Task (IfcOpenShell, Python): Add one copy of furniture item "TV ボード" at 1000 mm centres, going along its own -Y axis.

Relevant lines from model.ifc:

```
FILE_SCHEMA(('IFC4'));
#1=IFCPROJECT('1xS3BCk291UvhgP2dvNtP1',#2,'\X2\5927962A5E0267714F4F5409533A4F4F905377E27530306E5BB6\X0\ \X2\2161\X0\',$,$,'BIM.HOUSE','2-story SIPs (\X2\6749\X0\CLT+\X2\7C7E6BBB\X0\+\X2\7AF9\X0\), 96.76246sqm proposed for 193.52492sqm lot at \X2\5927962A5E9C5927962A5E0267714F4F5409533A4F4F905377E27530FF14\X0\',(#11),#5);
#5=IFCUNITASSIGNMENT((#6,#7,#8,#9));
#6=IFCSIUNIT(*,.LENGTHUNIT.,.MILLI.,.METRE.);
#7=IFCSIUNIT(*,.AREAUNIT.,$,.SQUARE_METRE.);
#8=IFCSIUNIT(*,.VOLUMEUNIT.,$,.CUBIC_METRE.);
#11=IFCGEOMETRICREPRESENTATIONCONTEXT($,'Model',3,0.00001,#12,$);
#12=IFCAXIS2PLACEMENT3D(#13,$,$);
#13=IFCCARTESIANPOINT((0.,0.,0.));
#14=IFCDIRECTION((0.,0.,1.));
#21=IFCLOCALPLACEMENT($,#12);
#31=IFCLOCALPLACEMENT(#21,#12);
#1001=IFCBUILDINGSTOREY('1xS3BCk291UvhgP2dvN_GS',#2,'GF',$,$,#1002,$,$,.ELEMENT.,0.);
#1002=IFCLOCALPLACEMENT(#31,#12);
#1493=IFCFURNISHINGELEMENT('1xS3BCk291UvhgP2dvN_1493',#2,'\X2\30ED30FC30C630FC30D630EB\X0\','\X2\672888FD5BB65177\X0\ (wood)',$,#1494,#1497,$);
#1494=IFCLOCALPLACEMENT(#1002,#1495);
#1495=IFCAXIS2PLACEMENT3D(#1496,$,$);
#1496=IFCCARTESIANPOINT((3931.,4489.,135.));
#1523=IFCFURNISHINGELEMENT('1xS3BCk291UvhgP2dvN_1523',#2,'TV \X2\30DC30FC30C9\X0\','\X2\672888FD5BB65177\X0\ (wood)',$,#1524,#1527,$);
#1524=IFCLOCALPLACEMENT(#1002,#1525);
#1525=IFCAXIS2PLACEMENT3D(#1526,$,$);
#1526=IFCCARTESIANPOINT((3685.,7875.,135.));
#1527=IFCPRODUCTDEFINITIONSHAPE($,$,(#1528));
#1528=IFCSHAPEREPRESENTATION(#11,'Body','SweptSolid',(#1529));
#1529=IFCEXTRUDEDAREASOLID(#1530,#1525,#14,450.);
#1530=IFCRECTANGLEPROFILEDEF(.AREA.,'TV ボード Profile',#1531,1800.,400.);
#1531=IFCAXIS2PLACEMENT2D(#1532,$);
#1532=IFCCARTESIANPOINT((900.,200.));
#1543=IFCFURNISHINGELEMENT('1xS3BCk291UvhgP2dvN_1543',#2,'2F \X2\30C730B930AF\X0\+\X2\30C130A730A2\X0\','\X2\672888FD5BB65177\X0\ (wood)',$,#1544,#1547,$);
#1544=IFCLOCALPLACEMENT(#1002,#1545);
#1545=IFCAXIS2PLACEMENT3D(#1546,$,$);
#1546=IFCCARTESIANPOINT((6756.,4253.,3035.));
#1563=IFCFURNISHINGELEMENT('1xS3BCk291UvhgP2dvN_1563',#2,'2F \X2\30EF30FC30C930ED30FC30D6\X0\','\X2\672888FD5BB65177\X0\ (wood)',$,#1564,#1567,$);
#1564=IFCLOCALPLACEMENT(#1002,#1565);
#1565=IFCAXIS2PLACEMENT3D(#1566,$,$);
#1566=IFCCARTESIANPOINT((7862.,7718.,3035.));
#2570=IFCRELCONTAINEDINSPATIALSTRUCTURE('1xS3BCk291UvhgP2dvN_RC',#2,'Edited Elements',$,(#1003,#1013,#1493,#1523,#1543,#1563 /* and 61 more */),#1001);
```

```python
import ifcopenshell
import ifcopenshell.api.geometry
import ifcopenshell.api.root
import ifcopenshell.util.element
import ifcopenshell.util.placement
import ifcopenshell.util.unit

model = ifcopenshell.open("model.ifc")
unit_scale = ifcopenshell.util.unit.calculate_unit_scale(model)


def reuse_history(source, copy):
    """copy_class also copies each property set's owner history, people and application; keep the originals."""
    for rel in copy.IsDefinedBy:
        if rel.is_a("IfcRelDefinesByProperties") and (history := rel.RelatingPropertyDefinition.OwnerHistory):
            rel.RelatingPropertyDefinition.OwnerHistory = source.OwnerHistory
            ifcopenshell.util.element.remove_deep2(model, history)


source = model.by_guid("1xS3BCk291UvhgP2dvN_1523")
base = ifcopenshell.util.placement.get_local_placement(source.ObjectPlacement)
step = -base[:3, 1] * 1 / unit_scale

for i in range(1, 2):
    copy = ifcopenshell.api.root.copy_class(model, product=source)
    copy.Representation = ifcopenshell.util.element.copy_deep(
        model, source.Representation, exclude=["IfcGeometricRepresentationContext", "IfcRepresentationMap"]
    )
    reuse_history(source, copy)
    matrix = base.copy()
    matrix[:3, 3] += i * step
    print("added at", matrix[:3, 3].round(3) + 0.0)
    ifcopenshell.api.geometry.edit_object_placement(model, product=copy, matrix=matrix, is_si=False)

model.write("model_rev.ifc")
```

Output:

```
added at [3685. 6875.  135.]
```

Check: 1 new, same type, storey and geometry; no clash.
